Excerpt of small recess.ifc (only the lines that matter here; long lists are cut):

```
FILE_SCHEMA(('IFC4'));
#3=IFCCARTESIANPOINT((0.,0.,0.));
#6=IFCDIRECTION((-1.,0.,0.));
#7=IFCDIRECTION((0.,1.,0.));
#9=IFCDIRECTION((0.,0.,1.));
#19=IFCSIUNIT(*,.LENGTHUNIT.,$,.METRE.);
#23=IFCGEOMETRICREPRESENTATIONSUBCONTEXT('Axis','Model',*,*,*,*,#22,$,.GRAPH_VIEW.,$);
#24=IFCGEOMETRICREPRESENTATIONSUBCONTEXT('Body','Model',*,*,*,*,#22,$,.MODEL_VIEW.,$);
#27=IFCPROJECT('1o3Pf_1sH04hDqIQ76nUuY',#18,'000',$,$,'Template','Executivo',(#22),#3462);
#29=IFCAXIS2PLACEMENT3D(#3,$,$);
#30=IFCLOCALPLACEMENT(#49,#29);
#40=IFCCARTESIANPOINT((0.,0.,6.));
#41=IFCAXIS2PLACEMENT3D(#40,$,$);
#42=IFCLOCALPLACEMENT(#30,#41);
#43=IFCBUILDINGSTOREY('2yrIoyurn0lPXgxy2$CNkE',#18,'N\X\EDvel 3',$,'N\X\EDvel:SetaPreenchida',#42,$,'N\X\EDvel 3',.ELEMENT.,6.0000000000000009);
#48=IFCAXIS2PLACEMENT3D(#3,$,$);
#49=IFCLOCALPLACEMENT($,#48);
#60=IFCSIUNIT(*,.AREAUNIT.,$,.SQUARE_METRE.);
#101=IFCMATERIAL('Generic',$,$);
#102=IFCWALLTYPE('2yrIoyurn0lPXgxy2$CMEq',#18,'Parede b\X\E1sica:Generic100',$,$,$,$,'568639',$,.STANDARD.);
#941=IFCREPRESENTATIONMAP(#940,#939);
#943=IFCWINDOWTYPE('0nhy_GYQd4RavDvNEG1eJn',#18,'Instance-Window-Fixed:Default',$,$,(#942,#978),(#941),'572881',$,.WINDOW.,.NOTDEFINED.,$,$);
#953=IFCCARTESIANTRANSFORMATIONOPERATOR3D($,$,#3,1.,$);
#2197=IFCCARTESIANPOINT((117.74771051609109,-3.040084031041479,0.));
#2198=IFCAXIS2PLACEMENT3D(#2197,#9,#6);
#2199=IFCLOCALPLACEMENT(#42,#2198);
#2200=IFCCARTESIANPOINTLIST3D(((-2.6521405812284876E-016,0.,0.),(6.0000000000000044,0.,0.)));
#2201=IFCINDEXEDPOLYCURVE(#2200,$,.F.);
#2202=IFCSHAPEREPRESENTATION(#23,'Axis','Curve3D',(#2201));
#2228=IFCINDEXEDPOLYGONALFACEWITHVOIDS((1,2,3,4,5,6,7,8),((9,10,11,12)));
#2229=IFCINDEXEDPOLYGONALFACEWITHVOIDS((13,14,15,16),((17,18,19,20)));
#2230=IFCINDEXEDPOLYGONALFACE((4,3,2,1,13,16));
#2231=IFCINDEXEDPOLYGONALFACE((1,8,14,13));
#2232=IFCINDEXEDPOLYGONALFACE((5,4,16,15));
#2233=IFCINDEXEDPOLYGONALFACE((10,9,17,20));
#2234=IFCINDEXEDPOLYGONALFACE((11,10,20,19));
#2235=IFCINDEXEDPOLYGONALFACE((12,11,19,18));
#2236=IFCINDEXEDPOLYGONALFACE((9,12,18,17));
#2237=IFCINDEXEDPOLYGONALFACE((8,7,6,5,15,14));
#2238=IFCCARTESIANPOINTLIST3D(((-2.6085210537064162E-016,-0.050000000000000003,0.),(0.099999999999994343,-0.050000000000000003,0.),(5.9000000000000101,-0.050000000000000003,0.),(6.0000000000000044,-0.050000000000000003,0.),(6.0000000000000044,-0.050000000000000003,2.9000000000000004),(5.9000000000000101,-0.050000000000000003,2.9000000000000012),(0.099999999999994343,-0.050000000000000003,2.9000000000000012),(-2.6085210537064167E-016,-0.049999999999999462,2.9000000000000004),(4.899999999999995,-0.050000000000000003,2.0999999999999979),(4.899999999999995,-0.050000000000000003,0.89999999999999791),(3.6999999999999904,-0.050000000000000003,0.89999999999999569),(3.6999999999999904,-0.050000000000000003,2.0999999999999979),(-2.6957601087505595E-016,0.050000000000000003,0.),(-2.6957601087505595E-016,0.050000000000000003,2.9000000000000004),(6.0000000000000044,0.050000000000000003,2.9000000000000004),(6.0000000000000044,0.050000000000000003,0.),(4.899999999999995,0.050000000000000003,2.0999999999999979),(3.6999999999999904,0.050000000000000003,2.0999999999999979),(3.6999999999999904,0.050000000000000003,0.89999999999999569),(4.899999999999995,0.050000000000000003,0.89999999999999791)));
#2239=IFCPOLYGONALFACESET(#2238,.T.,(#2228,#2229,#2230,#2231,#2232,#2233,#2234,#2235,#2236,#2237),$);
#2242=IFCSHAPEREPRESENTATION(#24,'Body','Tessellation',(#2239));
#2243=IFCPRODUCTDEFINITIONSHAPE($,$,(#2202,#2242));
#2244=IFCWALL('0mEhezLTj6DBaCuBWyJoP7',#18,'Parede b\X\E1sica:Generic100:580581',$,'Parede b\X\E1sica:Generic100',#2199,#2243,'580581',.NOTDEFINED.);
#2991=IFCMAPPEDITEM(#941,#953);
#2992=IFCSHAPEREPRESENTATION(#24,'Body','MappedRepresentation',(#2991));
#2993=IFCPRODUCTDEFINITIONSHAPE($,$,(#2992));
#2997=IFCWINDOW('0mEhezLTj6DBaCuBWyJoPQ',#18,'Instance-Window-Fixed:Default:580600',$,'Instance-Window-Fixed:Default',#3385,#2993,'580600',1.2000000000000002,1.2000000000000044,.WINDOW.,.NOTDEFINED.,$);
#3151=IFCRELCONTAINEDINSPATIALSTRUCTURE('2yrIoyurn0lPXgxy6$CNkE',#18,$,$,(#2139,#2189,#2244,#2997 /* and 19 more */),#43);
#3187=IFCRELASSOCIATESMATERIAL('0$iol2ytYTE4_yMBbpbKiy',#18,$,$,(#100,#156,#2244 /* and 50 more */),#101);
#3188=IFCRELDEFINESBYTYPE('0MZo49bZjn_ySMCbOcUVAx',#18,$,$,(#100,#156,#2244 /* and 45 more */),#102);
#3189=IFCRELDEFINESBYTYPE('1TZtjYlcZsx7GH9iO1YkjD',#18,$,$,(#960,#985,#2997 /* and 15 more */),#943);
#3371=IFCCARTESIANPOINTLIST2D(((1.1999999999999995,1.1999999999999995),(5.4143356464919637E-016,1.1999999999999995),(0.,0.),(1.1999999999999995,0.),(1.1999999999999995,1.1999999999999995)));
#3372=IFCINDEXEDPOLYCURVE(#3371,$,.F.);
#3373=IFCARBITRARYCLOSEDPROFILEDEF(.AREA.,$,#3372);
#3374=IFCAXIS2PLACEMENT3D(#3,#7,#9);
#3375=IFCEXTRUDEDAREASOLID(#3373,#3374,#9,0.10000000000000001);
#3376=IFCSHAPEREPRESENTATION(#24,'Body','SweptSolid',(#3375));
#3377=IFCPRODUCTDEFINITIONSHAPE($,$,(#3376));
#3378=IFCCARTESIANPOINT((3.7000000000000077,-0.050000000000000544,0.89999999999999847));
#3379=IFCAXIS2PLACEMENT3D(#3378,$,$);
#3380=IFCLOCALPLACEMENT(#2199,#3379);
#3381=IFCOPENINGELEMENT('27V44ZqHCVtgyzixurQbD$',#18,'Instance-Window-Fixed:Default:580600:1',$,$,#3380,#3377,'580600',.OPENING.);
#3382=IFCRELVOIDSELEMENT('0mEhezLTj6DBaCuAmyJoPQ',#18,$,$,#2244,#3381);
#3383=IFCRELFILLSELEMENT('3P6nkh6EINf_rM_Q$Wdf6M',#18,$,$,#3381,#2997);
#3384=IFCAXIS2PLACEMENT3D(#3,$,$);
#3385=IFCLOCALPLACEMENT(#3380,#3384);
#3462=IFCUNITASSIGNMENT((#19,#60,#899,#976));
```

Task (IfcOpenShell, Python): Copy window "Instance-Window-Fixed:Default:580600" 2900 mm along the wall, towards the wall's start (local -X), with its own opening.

```python
import ifcopenshell
import ifcopenshell.api.feature
import ifcopenshell.api.geometry
import ifcopenshell.api.root
import ifcopenshell.geom
import ifcopenshell.util.element
import ifcopenshell.util.placement
import ifcopenshell.util.shape
import ifcopenshell.util.unit

model = ifcopenshell.open("small recess.ifc")
unit_scale = ifcopenshell.util.unit.calculate_unit_scale(model)
settings = ifcopenshell.geom.settings()


def volume(element):
    """Net volume in cubic metres, openings subtracted."""
    shape = ifcopenshell.geom.create_shape(settings, element)
    return ifcopenshell.util.shape.get_volume(shape.geometry)


def reuse_history(source, copy):
    """copy_class also copies each property set's owner history, people and application; keep the originals."""
    for rel in copy.IsDefinedBy:
        if rel.is_a("IfcRelDefinesByProperties") and (history := rel.RelatingPropertyDefinition.OwnerHistory):
            rel.RelatingPropertyDefinition.OwnerHistory = source.OwnerHistory
            ifcopenshell.util.element.remove_deep2(model, history)


window = model.by_id(2997)
opening = window.FillsVoids[0].RelatingOpeningElement
wall = opening.VoidsElements[0].RelatingBuildingElement
before = volume(wall)
shift = ifcopenshell.util.placement.get_local_placement(wall.ObjectPlacement)[:3, 0] * -2.9 / unit_scale

# copy_class copies the void relationship, type, container and properties, but no geometry.
new_opening = ifcopenshell.api.root.copy_class(model, product=opening)
new_opening.Representation = ifcopenshell.util.element.copy_deep(
    model, opening.Representation, exclude=["IfcGeometricRepresentationContext", "IfcRepresentationMap"]
)
new_opening.Name = "Instance-Window-Fixed:Default"
new_opening.Tag = None
new_window = ifcopenshell.api.root.copy_class(model, product=window)
new_window.Representation = ifcopenshell.util.element.copy_deep(
    model, window.Representation, exclude=["IfcGeometricRepresentationContext", "IfcRepresentationMap"]
)
new_window.Name = "Instance-Window-Fixed:Default"
new_window.Tag = None
reuse_history(window, new_window)
ifcopenshell.api.feature.add_filling(model, opening=new_opening, element=new_window)

for old, new in ((opening, new_opening), (window, new_window)):
    matrix = ifcopenshell.util.placement.get_local_placement(old.ObjectPlacement)
    matrix[:3, 3] += shift
    ifcopenshell.api.geometry.edit_object_placement(model, product=new, matrix=matrix, is_si=False)

after = volume(wall)

print(f"wall volume {before:.3f} -> {after:.3f} m3")

model.write("small recess_edited.ifc")
```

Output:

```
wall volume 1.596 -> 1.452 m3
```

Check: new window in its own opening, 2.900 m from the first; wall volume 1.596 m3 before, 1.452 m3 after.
